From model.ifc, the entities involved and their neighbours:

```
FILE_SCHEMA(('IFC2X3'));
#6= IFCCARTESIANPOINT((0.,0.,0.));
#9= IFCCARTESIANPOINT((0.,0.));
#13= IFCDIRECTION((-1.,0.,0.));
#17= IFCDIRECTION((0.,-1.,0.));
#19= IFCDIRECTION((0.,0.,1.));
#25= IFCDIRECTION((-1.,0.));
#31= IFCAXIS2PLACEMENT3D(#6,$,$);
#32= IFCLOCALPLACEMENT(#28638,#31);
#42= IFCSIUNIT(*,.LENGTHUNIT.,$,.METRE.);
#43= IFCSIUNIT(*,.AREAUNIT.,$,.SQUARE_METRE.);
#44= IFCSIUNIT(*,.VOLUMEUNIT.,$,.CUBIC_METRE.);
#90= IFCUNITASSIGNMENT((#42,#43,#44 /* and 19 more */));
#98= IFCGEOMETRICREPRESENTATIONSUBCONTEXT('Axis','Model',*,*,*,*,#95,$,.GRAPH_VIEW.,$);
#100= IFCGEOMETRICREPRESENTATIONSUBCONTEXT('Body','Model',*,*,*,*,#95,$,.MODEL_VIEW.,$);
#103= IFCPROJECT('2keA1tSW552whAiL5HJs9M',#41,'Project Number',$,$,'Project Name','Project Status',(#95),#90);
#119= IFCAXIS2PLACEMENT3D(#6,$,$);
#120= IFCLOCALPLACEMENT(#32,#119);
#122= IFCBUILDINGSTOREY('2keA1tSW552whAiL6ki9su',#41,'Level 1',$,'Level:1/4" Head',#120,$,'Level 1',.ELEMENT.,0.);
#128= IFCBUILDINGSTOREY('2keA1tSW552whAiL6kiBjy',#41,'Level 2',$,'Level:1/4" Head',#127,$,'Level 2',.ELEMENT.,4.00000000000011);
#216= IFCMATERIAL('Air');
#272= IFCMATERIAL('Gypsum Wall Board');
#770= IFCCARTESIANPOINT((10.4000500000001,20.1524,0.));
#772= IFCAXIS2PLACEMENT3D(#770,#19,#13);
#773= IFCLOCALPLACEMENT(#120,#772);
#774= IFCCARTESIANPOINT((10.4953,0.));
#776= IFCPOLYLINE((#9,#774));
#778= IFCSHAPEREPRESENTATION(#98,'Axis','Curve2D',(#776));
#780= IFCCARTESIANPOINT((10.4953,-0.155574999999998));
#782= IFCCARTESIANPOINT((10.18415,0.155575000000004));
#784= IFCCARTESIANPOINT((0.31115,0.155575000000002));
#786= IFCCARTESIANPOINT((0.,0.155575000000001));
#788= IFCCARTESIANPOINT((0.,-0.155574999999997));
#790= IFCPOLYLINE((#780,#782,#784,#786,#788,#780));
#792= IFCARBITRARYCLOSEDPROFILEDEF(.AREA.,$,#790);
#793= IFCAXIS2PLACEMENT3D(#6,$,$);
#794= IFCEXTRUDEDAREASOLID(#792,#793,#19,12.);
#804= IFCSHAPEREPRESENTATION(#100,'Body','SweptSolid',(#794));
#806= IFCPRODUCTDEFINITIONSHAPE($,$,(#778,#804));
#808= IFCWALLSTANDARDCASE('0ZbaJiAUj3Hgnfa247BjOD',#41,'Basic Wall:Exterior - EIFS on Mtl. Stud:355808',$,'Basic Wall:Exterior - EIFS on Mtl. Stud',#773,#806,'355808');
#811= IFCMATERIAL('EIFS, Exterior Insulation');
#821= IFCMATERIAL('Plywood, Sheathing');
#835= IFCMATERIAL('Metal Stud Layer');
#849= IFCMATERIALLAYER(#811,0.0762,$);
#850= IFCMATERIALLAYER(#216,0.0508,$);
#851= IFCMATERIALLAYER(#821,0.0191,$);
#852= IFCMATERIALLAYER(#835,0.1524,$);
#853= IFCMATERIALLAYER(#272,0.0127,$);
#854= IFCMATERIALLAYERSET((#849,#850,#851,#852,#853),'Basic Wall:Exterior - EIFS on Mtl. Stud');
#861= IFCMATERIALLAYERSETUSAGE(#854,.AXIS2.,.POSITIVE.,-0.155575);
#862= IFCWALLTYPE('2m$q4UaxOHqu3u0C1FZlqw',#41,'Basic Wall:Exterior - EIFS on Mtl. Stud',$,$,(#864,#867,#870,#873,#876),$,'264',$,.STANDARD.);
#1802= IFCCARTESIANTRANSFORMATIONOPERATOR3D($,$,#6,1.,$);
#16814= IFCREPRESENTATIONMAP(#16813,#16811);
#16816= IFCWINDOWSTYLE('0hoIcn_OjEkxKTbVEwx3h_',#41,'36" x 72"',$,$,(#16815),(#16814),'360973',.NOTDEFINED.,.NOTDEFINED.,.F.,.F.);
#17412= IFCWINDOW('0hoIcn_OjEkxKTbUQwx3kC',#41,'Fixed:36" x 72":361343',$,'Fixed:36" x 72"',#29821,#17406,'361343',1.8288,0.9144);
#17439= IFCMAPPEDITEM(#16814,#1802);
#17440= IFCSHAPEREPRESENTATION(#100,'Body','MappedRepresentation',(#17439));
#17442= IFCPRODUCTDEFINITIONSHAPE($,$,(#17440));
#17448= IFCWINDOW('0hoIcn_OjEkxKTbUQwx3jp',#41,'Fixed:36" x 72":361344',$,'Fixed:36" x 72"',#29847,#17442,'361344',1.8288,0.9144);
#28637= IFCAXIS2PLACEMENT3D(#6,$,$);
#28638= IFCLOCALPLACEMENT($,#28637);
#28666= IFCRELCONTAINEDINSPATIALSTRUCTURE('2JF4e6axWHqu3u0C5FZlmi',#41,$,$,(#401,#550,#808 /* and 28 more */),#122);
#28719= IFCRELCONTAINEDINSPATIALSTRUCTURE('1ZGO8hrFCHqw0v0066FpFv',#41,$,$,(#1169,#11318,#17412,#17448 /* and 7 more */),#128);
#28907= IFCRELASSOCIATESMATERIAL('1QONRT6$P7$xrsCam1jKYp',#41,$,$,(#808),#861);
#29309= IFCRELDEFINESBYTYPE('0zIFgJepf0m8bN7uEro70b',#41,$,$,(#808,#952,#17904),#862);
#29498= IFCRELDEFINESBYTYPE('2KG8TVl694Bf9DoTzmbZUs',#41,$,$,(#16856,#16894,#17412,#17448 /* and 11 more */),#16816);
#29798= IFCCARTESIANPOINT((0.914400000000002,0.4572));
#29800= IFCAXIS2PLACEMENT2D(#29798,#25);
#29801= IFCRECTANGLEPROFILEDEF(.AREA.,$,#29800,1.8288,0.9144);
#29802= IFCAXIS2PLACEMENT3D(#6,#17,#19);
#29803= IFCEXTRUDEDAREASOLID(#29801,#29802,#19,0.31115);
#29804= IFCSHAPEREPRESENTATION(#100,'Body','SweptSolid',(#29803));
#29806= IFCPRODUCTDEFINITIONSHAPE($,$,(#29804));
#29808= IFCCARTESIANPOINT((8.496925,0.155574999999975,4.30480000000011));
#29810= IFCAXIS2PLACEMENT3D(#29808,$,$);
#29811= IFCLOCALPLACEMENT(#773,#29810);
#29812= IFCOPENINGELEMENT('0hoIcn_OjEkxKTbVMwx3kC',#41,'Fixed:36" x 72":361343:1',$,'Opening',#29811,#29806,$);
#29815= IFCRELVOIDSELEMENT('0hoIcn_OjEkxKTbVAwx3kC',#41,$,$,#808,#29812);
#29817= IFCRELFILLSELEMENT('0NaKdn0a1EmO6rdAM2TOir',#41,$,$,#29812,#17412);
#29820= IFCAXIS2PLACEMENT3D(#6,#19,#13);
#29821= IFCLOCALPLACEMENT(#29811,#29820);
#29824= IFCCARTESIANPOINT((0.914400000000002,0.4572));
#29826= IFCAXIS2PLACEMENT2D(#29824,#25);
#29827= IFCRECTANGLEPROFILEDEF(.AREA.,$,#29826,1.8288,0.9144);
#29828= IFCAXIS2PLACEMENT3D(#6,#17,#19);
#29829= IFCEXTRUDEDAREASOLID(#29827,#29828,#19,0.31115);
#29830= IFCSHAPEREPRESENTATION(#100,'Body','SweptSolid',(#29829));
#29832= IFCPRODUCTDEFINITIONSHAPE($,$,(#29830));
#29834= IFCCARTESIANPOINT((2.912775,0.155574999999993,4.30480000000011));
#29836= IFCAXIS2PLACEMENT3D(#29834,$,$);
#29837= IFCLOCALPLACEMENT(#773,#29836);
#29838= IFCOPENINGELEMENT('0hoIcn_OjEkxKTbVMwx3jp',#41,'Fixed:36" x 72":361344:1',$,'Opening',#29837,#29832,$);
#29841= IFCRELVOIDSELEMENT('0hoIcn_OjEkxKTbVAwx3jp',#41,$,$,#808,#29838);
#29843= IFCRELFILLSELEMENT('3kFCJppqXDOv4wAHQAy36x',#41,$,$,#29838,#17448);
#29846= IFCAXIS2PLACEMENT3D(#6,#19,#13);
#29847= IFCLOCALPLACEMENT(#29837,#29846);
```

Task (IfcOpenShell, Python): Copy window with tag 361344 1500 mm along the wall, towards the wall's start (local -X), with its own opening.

```python
import ifcopenshell
import ifcopenshell.api.feature
import ifcopenshell.api.geometry
import ifcopenshell.api.root
import ifcopenshell.geom
import ifcopenshell.util.element
import ifcopenshell.util.placement
import ifcopenshell.util.shape

model = ifcopenshell.open("model.ifc")
settings = ifcopenshell.geom.settings()


def volume(element):
    """Net volume in cubic metres, openings subtracted."""
    shape = ifcopenshell.geom.create_shape(settings, element)
    return ifcopenshell.util.shape.get_volume(shape.geometry)


def reuse_history(source, copy):
    """copy_class also copies each property set's owner history, people and application; keep the originals."""
    for rel in copy.IsDefinedBy:
        if rel.is_a("IfcRelDefinesByProperties") and (history := rel.RelatingPropertyDefinition.OwnerHistory):
            rel.RelatingPropertyDefinition.OwnerHistory = source.OwnerHistory
            ifcopenshell.util.element.remove_deep2(model, history)


window = model.by_guid("0hoIcn_OjEkxKTbUQwx3jp")
opening = window.FillsVoids[0].RelatingOpeningElement
wall = opening.VoidsElements[0].RelatingBuildingElement
before = volume(wall)
shift = ifcopenshell.util.placement.get_local_placement(wall.ObjectPlacement)[:3, 0] * -1.5

# copy_class copies the void relationship, type, container and properties, but no geometry.
new_opening = ifcopenshell.api.root.copy_class(model, product=opening)
new_opening.Representation = ifcopenshell.util.element.copy_deep(
    model, opening.Representation, exclude=["IfcGeometricRepresentationContext", "IfcRepresentationMap"]
)
new_opening.Name = 'Fixed:36" x 72"'
new_window = ifcopenshell.api.root.copy_class(model, product=window)
new_window.Representation = ifcopenshell.util.element.copy_deep(
    model, window.Representation, exclude=["IfcGeometricRepresentationContext", "IfcRepresentationMap"]
)
new_window.Name = 'Fixed:36" x 72"'
new_window.Tag = None
reuse_history(window, new_window)
fills = ifcopenshell.api.feature.add_filling(model, opening=new_opening, element=new_window)
fills.OwnerHistory = new_window.OwnerHistory  # required in IFC2X3

for old, new in ((opening, new_opening), (window, new_window)):
    matrix = ifcopenshell.util.placement.get_local_placement(old.ObjectPlacement)
    matrix[:3, 3] += shift
    ifcopenshell.api.geometry.edit_object_placement(model, product=new, matrix=matrix, is_si=False)

after = volume(wall)

print(f"wall volume {before:.3f} -> {after:.3f} m3")

model.write("model_edited.ifc")
```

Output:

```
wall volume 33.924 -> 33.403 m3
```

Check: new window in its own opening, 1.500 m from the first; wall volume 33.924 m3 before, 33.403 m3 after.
